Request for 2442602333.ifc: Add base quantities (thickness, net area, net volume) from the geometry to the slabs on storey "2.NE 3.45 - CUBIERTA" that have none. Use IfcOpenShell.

First a look at what the model holds.

```python
import ifcopenshell
import ifcopenshell.util.element
import ifcopenshell.util.unit

model = ifcopenshell.open("2442602333.ifc")
print(model.schema)
for unit_type in ("LENGTHUNIT", "AREAUNIT", "VOLUMEUNIT"):
    print(unit_type, ifcopenshell.util.unit.calculate_unit_scale(model, unit_type))
storey = next(s for s in model.by_type("IfcBuildingStorey") if s.Name == "2.NE 3.45 - CUBIERTA")
slabs = [e for e in ifcopenshell.util.element.get_decomposition(storey) if e.is_a("IfcSlab")]
for e in sorted(slabs, key=lambda e: e.id()):
    print(e.id(), e.is_a(), e.Name, list(ifcopenshell.util.element.get_psets(e, qtos_only=True)), sep=" | ")
```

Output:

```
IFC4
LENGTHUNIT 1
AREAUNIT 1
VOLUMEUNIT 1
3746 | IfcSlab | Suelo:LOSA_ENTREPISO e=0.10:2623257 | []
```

```python
import ifcopenshell
import ifcopenshell.api.pset
import ifcopenshell.geom
import ifcopenshell.util.element
import ifcopenshell.util.shape
import ifcopenshell.util.unit

model = ifcopenshell.open("2442602333.ifc")
unit_scale = ifcopenshell.util.unit.calculate_unit_scale(model)
area_scale = ifcopenshell.util.unit.calculate_unit_scale(model, "AREAUNIT")
volume_scale = ifcopenshell.util.unit.calculate_unit_scale(model, "VOLUMEUNIT")
settings = ifcopenshell.geom.settings()

storey = next(s for s in model.by_type("IfcBuildingStorey") if s.Name == "2.NE 3.45 - CUBIERTA")
slabs = [e for e in ifcopenshell.util.element.get_decomposition(storey) if e.is_a("IfcSlab")]

for e in sorted(slabs, key=lambda e: e.id()):
    if ifcopenshell.util.element.get_psets(e, qtos_only=True, should_inherit=False):
        continue
    # Geometry comes back in metres, in the element's own axes.
    shape = ifcopenshell.geom.create_shape(settings, e)
    values = {
        "Width": ifcopenshell.util.shape.get_z(shape.geometry) / unit_scale,
        "NetArea": ifcopenshell.util.shape.get_footprint_area(shape.geometry) / area_scale,
        "NetVolume": ifcopenshell.util.shape.get_volume(shape.geometry) / volume_scale,
    }
    qto = ifcopenshell.api.pset.add_qto(model, product=e, name="Qto_SlabBaseQuantities")
    ifcopenshell.api.pset.edit_qto(model, qto=qto, properties=values)
    print(e.id(), {k: round(v, 3) for k, v in values.items()})

model.write("2442602333_updated.ifc")
```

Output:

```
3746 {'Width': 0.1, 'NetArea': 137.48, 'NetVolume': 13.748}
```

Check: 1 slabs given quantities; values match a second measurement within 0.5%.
